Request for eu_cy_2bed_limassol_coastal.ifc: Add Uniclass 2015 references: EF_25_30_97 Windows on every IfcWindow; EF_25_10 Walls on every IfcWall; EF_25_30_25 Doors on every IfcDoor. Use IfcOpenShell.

First a look at what the model holds.

```python
import ifcopenshell

model = ifcopenshell.open("eu_cy_2bed_limassol_coastal.ifc")
print(model.schema)
print("classifications:", [c.Name for c in model.by_type("IfcClassification")])
for ifc_class in ("IfcDoor", "IfcRoof", "IfcStair", "IfcWall", "IfcWindow"):
    print(ifc_class, len(model.by_type(ifc_class)))
```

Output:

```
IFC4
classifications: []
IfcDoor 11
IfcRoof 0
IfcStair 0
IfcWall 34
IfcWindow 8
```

```python
import ifcopenshell
import ifcopenshell.api.classification

model = ifcopenshell.open("eu_cy_2bed_limassol_coastal.ifc")

system = ifcopenshell.api.classification.add_classification(model, classification="Uniclass 2015")

codes = {
    "IfcWindow": ("EF_25_30_97", "Windows"),
    "IfcWall": ("EF_25_10", "Walls"),
    "IfcDoor": ("EF_25_30_25", "Doors"),
}
for ifc_class, (code, name) in codes.items():
    products = model.by_type(ifc_class)
    ifcopenshell.api.classification.add_reference(
        model, products=products, classification=system, identification=code, name=name
    )
    print(code, len(products))

model.write("eu_cy_2bed_limassol_coastal_edited.ifc")
```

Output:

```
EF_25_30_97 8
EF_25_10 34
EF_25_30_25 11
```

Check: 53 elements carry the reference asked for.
